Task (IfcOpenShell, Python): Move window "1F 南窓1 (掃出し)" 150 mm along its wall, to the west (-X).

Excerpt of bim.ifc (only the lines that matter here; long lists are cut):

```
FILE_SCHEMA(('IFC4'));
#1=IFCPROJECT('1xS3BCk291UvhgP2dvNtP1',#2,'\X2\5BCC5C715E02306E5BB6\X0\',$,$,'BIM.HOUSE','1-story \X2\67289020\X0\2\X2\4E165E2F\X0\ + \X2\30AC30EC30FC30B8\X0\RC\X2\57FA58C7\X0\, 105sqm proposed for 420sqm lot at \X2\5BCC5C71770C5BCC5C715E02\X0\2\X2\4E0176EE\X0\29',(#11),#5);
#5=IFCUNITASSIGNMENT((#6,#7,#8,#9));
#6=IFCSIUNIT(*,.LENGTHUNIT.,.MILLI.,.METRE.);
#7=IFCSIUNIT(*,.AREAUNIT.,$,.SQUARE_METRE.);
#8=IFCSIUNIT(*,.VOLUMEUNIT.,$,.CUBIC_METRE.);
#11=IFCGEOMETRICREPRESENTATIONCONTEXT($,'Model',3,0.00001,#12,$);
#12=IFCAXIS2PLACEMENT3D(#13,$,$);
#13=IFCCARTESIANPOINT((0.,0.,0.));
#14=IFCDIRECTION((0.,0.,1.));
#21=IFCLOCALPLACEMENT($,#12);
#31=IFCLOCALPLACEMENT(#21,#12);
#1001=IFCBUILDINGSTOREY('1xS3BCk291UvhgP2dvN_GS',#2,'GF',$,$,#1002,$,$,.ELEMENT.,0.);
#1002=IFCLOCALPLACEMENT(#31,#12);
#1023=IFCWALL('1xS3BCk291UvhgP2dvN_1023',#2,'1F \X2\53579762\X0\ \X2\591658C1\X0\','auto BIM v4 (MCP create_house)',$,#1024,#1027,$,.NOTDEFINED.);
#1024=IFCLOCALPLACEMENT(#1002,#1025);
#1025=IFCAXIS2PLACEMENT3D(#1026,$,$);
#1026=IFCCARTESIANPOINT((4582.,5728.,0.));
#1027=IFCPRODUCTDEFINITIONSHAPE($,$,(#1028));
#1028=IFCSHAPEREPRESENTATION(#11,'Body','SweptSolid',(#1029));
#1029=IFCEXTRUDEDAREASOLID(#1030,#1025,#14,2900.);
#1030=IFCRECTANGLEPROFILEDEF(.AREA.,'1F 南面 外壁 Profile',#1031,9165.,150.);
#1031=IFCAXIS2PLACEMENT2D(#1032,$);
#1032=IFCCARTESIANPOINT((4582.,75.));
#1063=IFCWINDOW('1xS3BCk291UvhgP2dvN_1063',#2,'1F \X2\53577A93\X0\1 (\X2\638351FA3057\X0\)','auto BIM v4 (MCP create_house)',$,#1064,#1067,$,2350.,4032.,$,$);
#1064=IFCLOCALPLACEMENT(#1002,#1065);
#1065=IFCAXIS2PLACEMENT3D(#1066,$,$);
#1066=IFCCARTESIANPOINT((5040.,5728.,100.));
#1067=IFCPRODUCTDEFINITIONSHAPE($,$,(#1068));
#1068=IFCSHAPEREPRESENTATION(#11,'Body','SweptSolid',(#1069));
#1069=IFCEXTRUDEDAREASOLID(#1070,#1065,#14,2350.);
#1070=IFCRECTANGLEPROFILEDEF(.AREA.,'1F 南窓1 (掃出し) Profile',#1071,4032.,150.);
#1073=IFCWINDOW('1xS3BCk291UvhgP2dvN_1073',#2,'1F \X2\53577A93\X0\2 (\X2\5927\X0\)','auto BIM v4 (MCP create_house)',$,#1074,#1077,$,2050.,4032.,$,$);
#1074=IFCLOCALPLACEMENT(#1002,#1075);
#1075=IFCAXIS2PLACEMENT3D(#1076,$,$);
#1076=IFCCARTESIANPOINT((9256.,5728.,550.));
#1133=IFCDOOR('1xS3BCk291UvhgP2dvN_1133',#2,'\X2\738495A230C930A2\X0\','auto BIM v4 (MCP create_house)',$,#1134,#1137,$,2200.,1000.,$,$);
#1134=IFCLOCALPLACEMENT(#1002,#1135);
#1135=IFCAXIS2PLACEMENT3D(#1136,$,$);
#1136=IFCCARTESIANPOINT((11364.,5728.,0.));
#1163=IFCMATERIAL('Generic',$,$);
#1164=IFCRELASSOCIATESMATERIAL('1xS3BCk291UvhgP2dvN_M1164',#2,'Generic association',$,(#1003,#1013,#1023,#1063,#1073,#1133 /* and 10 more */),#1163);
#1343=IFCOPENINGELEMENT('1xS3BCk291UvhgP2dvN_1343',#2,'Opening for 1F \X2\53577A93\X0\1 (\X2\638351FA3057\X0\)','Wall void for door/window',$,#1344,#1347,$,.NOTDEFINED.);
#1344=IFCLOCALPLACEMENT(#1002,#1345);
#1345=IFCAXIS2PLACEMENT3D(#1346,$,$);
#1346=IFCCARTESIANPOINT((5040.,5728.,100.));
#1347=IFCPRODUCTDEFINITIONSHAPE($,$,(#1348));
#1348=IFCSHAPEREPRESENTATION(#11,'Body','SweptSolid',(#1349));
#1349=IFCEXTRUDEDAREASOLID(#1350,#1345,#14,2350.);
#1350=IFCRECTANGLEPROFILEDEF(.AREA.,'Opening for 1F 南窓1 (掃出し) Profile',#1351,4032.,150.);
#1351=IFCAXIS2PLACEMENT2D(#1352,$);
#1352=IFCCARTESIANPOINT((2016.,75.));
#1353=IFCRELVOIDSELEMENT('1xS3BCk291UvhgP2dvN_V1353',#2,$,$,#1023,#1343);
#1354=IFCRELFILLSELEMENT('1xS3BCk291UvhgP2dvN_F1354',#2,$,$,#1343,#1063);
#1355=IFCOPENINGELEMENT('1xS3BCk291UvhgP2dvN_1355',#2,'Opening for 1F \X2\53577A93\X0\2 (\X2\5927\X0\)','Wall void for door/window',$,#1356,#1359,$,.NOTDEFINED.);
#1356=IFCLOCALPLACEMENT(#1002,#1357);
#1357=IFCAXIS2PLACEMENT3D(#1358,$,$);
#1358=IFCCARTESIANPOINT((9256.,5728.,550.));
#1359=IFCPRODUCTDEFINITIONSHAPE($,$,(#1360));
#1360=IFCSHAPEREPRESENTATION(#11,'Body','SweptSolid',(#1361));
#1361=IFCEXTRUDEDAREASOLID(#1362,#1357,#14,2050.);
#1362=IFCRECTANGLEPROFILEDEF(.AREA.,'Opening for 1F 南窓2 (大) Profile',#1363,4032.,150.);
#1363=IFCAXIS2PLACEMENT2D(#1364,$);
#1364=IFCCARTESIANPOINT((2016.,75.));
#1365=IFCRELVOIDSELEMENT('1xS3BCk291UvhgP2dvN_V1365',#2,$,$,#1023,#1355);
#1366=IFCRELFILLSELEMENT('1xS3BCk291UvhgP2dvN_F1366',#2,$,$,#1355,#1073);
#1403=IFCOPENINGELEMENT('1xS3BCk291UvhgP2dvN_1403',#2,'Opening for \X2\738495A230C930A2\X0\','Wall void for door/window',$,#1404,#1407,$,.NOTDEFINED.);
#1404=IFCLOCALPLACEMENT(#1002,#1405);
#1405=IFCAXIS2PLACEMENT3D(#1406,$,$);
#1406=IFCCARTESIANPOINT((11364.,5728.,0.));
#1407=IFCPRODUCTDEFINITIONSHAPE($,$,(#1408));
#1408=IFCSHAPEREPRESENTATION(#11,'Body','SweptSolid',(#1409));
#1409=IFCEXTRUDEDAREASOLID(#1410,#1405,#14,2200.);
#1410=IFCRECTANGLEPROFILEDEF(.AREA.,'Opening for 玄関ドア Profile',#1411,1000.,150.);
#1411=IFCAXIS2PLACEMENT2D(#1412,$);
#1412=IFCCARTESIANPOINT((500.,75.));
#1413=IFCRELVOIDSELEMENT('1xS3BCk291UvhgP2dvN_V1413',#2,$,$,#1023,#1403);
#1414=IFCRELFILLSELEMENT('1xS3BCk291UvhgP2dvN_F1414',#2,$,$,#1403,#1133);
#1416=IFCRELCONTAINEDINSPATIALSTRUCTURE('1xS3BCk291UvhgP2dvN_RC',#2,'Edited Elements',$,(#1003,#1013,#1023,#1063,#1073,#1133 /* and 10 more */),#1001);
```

```python
import ifcopenshell
import ifcopenshell.api.geometry
import ifcopenshell.util.placement
import ifcopenshell.util.unit

model = ifcopenshell.open("bim.ifc")
unit_scale = ifcopenshell.util.unit.calculate_unit_scale(model)

window = model.by_guid("1xS3BCk291UvhgP2dvN_1063")
opening = window.FillsVoids[0].RelatingOpeningElement
wall = opening.VoidsElements[0].RelatingBuildingElement

wall_matrix = ifcopenshell.util.placement.get_local_placement(wall.ObjectPlacement)
shift = wall_matrix[:3, 0] * -0.15 / unit_scale
before = ifcopenshell.util.placement.get_local_placement(window.ObjectPlacement)[:3, 3].copy()

# The window is not placed relative to its opening, so move both.
for product in (opening, window):
    matrix = ifcopenshell.util.placement.get_local_placement(product.ObjectPlacement)
    matrix[:3, 3] += shift
    ifcopenshell.api.geometry.edit_object_placement(model, product=product, matrix=matrix, is_si=False)

after = ifcopenshell.util.placement.get_local_placement(window.ObjectPlacement)[:3, 3]
print("window moved by", (after - before).round(3) + 0.0)

model.write("bim_edited.ifc")
```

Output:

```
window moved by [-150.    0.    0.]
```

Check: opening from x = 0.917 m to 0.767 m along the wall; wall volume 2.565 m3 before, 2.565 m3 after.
